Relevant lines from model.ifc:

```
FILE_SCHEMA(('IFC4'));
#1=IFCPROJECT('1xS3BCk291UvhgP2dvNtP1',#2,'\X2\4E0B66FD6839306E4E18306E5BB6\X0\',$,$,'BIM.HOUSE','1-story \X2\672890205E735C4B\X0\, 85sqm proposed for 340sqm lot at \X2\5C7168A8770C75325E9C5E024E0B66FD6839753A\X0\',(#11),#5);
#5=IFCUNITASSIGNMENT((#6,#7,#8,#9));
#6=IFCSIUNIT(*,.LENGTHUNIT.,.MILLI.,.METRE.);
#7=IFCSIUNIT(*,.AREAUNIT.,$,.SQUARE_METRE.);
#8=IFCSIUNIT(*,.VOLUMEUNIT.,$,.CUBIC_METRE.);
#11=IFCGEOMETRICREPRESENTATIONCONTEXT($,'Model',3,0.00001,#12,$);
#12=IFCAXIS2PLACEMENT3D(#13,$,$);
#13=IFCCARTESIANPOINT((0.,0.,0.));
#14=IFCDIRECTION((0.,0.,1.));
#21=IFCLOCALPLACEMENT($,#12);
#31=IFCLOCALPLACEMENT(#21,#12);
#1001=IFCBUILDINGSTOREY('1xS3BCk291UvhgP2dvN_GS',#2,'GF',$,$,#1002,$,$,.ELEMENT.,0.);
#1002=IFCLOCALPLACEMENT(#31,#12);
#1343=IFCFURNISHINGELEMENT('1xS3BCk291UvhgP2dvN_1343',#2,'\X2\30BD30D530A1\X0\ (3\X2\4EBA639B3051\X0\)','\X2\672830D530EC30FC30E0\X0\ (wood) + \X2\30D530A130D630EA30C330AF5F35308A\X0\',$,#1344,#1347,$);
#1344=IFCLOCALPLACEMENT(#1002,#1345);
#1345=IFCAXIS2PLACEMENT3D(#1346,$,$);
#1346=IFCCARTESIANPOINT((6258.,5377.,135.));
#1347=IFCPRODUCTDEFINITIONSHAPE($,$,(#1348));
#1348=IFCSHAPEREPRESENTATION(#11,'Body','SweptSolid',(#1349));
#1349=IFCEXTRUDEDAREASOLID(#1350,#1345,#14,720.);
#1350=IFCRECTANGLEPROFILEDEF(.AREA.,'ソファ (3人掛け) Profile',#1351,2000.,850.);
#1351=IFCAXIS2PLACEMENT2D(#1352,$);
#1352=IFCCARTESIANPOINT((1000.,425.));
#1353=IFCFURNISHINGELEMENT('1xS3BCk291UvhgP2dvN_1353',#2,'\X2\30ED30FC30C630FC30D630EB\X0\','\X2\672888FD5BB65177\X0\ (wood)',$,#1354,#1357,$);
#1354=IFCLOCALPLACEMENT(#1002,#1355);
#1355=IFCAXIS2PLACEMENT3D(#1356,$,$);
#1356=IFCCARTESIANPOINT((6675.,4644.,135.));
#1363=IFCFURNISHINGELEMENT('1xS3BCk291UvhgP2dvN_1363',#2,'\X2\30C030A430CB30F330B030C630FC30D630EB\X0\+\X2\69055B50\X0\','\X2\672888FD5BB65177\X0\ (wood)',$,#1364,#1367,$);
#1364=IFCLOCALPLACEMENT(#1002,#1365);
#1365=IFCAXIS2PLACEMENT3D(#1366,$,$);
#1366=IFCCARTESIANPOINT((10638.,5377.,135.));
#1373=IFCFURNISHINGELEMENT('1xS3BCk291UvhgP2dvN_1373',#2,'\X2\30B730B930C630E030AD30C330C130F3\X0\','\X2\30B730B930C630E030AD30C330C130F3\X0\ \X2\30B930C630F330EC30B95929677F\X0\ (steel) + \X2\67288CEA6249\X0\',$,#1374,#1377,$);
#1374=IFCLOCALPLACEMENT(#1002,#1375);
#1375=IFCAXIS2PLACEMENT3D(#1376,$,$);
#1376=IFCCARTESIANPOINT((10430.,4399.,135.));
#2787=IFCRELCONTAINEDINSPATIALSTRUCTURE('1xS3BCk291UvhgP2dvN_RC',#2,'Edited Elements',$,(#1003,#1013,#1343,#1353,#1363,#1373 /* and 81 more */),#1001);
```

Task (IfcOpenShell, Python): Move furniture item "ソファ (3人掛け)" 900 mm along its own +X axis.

```python
import ifcopenshell
import ifcopenshell.api.geometry
import ifcopenshell.util.placement

model = ifcopenshell.open("model.ifc")

item = model.by_id(1343)
matrix = ifcopenshell.util.placement.get_local_placement(item.ObjectPlacement)
matrix[:3, 3] += matrix[:3, 0] * 900.0
ifcopenshell.api.geometry.edit_object_placement(model, product=item, matrix=matrix, is_si=False)

print(ifcopenshell.util.placement.get_local_placement(item.ObjectPlacement).round(3) + 0.0)

model.write("model_v2.ifc")
```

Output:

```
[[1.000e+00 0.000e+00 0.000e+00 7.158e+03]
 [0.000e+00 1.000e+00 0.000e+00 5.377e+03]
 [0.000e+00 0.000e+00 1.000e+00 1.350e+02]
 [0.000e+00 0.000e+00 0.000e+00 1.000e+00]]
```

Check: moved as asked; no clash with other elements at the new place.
